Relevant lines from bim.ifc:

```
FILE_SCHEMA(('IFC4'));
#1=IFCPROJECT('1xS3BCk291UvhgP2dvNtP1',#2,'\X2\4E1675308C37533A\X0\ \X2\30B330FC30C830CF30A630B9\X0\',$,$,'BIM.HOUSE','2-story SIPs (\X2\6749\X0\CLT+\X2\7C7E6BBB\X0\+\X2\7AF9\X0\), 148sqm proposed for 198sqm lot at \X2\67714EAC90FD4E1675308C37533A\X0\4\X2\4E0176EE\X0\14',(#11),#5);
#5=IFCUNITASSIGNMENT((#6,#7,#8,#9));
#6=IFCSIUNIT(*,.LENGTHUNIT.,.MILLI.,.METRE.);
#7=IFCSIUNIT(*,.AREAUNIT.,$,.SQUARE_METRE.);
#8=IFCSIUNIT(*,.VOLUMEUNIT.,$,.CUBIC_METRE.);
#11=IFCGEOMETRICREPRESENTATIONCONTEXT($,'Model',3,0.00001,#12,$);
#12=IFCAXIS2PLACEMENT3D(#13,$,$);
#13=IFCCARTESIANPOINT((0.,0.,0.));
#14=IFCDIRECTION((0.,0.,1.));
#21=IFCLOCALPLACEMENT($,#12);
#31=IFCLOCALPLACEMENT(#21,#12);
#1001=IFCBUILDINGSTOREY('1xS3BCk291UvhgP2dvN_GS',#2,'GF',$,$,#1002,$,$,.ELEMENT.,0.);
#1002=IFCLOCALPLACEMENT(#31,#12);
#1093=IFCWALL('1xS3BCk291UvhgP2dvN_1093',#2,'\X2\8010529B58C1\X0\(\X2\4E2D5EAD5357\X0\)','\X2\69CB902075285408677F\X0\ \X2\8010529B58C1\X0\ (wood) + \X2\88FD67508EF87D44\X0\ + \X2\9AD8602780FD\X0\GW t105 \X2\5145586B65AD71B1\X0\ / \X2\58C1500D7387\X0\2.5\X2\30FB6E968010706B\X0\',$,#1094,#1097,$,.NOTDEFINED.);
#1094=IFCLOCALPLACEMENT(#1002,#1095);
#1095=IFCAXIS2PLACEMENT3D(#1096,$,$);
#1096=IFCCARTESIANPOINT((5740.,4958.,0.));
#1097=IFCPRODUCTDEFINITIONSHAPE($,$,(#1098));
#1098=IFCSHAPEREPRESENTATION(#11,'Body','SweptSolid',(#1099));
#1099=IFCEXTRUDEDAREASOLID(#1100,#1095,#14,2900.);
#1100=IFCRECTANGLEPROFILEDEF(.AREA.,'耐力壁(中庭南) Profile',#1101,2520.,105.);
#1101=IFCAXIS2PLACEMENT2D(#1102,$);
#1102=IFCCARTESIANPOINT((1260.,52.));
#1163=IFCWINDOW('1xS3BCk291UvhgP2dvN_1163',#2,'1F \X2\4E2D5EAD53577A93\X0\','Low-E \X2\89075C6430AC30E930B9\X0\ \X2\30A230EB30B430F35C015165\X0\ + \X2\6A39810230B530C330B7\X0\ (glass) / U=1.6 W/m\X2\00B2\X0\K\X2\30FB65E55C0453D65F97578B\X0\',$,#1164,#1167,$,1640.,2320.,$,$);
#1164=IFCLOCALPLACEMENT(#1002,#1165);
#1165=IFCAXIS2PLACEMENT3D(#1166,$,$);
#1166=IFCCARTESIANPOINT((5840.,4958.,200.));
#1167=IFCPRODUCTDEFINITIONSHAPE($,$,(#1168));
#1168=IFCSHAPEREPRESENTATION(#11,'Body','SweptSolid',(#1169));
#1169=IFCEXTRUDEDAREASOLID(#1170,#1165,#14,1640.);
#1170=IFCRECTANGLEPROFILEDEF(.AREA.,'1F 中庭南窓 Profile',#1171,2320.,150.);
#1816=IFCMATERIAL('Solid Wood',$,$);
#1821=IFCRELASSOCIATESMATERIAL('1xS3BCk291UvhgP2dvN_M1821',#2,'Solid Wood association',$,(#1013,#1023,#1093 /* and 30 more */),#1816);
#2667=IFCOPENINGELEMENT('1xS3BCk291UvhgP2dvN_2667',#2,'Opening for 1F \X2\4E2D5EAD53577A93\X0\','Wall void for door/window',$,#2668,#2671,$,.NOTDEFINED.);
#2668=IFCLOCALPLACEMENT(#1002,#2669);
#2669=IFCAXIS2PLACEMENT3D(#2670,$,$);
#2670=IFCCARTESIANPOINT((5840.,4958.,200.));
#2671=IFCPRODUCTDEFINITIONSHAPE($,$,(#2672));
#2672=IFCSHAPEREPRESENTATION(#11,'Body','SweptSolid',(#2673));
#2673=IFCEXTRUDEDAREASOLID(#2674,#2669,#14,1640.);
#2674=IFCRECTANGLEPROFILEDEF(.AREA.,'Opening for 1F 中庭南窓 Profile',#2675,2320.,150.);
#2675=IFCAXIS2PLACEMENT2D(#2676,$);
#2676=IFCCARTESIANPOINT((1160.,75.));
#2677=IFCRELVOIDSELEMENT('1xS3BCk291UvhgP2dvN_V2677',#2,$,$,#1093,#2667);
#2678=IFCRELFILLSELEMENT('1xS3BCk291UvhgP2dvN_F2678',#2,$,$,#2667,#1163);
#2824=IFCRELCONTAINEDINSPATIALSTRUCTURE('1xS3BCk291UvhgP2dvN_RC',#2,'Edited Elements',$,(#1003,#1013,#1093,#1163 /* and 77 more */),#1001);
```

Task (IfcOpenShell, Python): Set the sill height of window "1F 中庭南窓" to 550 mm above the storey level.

```python
import numpy as np
import ifcopenshell
import ifcopenshell.api.geometry
import ifcopenshell.geom
import ifcopenshell.util.element
import ifcopenshell.util.placement
import ifcopenshell.util.shape
import ifcopenshell.util.unit

model = ifcopenshell.open("bim.ifc")
unit_scale = ifcopenshell.util.unit.calculate_unit_scale(model)

window = model.by_id(1163)
opening = window.FillsVoids[0].RelatingOpeningElement
storey = ifcopenshell.util.element.get_container(window, ifc_class="IfcBuildingStorey")
level = ifcopenshell.util.placement.get_local_placement(storey.ObjectPlacement)[2, 3]

# The opening's origin need not be at the sill, so measure its lowest point.
shape = ifcopenshell.geom.create_shape(ifcopenshell.geom.settings(), opening)
bottom = ifcopenshell.util.shape.get_shape_bottom_elevation(shape, shape.geometry) / unit_scale
dz = level + 0.55 / unit_scale - bottom

shift = np.array([0.0, 0.0, dz])
# The window is not placed relative to its opening, so move both.
for product in (opening, window):
    matrix = ifcopenshell.util.placement.get_local_placement(product.ObjectPlacement)
    matrix[:3, 3] += shift
    ifcopenshell.api.geometry.edit_object_placement(model, product=product, matrix=matrix, is_si=False)

print(f"moved by {dz * unit_scale:+.3f} m")

model.write("bim_v2.ifc")
```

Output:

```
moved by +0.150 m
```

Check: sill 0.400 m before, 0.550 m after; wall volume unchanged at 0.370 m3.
